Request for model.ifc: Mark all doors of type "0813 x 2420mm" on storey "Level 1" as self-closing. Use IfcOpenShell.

First a look at what the model holds.

```python
import ifcopenshell
import ifcopenshell.util.element

model = ifcopenshell.open("model.ifc")
print(model.schema)
storey = next(s for s in model.by_type("IfcBuildingStorey") if s.Name == "Level 1")
doors = [e for e in ifcopenshell.util.element.get_decomposition(storey) if e.is_a("IfcDoor")]
seen = {}
for e in doors:
    element_type = ifcopenshell.util.element.get_type(e)
    key = (element_type.Name if element_type != e and element_type else None, ifcopenshell.util.element.get_pset(e, "Pset_DoorCommon", "SelfClosing"))
    seen[key] = seen.get(key, 0) + 1
for (name, value), count in sorted(seen.items(), key=str):
    print(count, "x", name, "|", value)
```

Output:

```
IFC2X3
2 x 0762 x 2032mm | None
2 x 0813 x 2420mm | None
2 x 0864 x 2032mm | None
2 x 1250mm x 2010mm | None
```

```python
import ifcopenshell
import ifcopenshell.api.pset
import ifcopenshell.util.element

model = ifcopenshell.open("model.ifc")

storey = next(s for s in model.by_type("IfcBuildingStorey") if s.Name == "Level 1")
doors = [e for e in ifcopenshell.util.element.get_decomposition(storey) if e.is_a("IfcDoor")]

count = 0
for e in doors:
    element_type = ifcopenshell.util.element.get_type(e)
    if element_type in (None, e) or element_type.Name != "0813 x 2420mm":
        continue
    # add_pset returns the element's existing set when there is one.
    pset = ifcopenshell.api.pset.add_pset(model, product=e, name="Pset_DoorCommon")
    ifcopenshell.api.pset.edit_pset(model, pset=pset, properties={"SelfClosing": True})
    count += 1

print(count, "doors updated")

model.write("model-out.ifc")
```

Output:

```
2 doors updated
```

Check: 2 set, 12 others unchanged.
